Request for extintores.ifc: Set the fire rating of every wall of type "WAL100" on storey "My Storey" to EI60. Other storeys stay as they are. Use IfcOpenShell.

First a look at what the model holds.

```python
import ifcopenshell
import ifcopenshell.util.element

model = ifcopenshell.open("extintores.ifc")
print(model.schema)
storey = next(s for s in model.by_type("IfcBuildingStorey") if s.Name == "My Storey")
walls = [e for e in ifcopenshell.util.element.get_decomposition(storey) if e.is_a("IfcWall")]
seen = {}
for e in walls:
    element_type = ifcopenshell.util.element.get_type(e)
    key = (element_type.Name if element_type != e and element_type else None, ifcopenshell.util.element.get_pset(e, "Pset_WallCommon", "FireRating"))
    seen[key] = seen.get(key, 0) + 1
for (name, value), count in sorted(seen.items(), key=str):
    print(count, "x", name, "|", value)
```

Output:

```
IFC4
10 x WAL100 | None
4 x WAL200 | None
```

```python
import ifcopenshell
import ifcopenshell.api.pset
import ifcopenshell.util.element

model = ifcopenshell.open("extintores.ifc")

storey = next(s for s in model.by_type("IfcBuildingStorey") if s.Name == "My Storey")
walls = [e for e in ifcopenshell.util.element.get_decomposition(storey) if e.is_a("IfcWall")]

count = 0
for e in walls:
    element_type = ifcopenshell.util.element.get_type(e)
    if element_type in (None, e) or element_type.Name != "WAL100":
        continue
    # add_pset returns the element's existing set when there is one.
    pset = ifcopenshell.api.pset.add_pset(model, product=e, name="Pset_WallCommon")
    ifcopenshell.api.pset.edit_pset(model, pset=pset, properties={"FireRating": "EI60"})
    count += 1

print(count, "walls updated")

model.write("extintores_v2.ifc")
```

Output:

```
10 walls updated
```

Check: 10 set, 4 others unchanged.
